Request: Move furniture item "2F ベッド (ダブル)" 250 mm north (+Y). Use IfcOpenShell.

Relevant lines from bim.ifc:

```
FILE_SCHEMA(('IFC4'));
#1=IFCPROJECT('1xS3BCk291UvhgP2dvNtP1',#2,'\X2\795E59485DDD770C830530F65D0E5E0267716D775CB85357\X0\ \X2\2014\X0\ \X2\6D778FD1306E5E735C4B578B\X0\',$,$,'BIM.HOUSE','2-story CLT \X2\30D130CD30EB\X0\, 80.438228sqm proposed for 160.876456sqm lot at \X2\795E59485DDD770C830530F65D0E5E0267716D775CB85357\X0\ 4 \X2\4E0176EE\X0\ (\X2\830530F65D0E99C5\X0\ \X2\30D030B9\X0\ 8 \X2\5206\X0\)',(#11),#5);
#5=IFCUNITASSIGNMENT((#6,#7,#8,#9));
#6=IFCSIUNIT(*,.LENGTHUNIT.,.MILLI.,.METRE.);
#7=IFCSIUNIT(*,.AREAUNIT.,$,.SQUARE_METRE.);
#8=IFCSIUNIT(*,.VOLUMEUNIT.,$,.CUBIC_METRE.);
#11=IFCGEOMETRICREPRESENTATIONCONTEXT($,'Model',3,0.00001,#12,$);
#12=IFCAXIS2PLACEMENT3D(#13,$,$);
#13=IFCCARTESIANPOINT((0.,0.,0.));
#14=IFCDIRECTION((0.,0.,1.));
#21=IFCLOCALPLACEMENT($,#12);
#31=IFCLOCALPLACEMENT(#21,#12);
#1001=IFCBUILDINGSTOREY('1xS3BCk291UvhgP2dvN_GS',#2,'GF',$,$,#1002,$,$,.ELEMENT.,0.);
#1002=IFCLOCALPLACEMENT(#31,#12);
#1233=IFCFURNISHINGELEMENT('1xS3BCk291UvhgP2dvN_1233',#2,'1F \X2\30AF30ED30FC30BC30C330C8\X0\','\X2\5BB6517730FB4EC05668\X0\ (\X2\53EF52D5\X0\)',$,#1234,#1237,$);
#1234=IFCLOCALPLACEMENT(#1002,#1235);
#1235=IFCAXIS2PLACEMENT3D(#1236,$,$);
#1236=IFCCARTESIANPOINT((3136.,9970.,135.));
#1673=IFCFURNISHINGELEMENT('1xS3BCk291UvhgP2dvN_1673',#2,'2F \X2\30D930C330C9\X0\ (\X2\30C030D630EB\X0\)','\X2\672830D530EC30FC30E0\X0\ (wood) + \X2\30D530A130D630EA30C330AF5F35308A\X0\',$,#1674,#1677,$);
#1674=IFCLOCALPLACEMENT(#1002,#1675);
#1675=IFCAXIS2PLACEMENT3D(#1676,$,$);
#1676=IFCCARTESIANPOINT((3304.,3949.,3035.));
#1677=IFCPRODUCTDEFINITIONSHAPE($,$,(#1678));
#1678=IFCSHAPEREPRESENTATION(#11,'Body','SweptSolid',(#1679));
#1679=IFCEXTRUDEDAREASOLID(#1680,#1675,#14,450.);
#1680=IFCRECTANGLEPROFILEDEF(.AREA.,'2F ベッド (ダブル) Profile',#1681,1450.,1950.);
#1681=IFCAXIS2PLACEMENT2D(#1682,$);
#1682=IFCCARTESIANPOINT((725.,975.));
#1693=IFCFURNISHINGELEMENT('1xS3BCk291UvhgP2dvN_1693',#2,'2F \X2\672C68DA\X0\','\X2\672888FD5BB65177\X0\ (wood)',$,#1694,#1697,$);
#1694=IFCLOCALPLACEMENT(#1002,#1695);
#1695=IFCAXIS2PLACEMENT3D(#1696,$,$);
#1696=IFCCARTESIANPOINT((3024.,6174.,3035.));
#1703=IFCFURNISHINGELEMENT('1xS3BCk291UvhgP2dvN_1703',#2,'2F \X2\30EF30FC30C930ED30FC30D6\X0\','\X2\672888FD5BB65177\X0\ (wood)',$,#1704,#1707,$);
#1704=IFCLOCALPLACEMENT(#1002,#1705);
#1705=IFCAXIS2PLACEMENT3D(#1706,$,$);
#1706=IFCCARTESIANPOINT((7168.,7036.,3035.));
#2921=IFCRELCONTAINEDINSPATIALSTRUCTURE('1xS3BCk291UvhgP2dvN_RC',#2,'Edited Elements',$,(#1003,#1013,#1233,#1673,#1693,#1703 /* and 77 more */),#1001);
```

```python
import ifcopenshell
import ifcopenshell.api.geometry
import ifcopenshell.util.placement
import ifcopenshell.util.unit

model = ifcopenshell.open("bim.ifc")
unit_scale = ifcopenshell.util.unit.calculate_unit_scale(model)

item = model.by_guid("1xS3BCk291UvhgP2dvN_1673")
matrix = ifcopenshell.util.placement.get_local_placement(item.ObjectPlacement)
matrix[1, 3] += 0.25 / unit_scale
ifcopenshell.api.geometry.edit_object_placement(model, product=item, matrix=matrix, is_si=False)

print(ifcopenshell.util.placement.get_local_placement(item.ObjectPlacement).round(3) + 0.0)

model.write("bim-out.ifc")
```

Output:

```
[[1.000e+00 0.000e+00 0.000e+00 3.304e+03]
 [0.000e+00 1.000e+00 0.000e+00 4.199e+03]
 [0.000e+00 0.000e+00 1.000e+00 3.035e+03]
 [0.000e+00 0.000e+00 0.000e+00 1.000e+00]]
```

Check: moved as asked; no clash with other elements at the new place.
